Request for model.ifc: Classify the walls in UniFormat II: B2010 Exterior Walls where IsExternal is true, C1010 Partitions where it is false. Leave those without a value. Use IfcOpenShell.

First a look at what the model holds.

```python
import ifcopenshell
import ifcopenshell.util.element

model = ifcopenshell.open("model.ifc")
print(model.schema)
print("classifications:", [c.Name for c in model.by_type("IfcClassification")])
values = [ifcopenshell.util.element.get_pset(e, "Pset_WallCommon", "IsExternal") for e in model.by_type("IfcWall")]
for value in (True, False, None):
    print("IsExternal", value, values.count(value))
```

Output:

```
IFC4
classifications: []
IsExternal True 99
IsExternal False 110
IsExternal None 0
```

```python
import ifcopenshell
import ifcopenshell.api.classification
import ifcopenshell.util.element

model = ifcopenshell.open("model.ifc")

system = ifcopenshell.api.classification.add_classification(model, classification="UniFormat II")

walls = model.by_type("IfcWall")
external = {e: ifcopenshell.util.element.get_pset(e, "Pset_WallCommon", "IsExternal") for e in walls}
for flag, code, name in ((True, "B2010", "Exterior Walls"), (False, "C1010", "Partitions")):
    products = [e for e in walls if external[e] is flag]
    ifcopenshell.api.classification.add_reference(
        model, products=products, classification=system, identification=code, name=name
    )
    print(code, len(products))

model.write("model_updated.ifc")
```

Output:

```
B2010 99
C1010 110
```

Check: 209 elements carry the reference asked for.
